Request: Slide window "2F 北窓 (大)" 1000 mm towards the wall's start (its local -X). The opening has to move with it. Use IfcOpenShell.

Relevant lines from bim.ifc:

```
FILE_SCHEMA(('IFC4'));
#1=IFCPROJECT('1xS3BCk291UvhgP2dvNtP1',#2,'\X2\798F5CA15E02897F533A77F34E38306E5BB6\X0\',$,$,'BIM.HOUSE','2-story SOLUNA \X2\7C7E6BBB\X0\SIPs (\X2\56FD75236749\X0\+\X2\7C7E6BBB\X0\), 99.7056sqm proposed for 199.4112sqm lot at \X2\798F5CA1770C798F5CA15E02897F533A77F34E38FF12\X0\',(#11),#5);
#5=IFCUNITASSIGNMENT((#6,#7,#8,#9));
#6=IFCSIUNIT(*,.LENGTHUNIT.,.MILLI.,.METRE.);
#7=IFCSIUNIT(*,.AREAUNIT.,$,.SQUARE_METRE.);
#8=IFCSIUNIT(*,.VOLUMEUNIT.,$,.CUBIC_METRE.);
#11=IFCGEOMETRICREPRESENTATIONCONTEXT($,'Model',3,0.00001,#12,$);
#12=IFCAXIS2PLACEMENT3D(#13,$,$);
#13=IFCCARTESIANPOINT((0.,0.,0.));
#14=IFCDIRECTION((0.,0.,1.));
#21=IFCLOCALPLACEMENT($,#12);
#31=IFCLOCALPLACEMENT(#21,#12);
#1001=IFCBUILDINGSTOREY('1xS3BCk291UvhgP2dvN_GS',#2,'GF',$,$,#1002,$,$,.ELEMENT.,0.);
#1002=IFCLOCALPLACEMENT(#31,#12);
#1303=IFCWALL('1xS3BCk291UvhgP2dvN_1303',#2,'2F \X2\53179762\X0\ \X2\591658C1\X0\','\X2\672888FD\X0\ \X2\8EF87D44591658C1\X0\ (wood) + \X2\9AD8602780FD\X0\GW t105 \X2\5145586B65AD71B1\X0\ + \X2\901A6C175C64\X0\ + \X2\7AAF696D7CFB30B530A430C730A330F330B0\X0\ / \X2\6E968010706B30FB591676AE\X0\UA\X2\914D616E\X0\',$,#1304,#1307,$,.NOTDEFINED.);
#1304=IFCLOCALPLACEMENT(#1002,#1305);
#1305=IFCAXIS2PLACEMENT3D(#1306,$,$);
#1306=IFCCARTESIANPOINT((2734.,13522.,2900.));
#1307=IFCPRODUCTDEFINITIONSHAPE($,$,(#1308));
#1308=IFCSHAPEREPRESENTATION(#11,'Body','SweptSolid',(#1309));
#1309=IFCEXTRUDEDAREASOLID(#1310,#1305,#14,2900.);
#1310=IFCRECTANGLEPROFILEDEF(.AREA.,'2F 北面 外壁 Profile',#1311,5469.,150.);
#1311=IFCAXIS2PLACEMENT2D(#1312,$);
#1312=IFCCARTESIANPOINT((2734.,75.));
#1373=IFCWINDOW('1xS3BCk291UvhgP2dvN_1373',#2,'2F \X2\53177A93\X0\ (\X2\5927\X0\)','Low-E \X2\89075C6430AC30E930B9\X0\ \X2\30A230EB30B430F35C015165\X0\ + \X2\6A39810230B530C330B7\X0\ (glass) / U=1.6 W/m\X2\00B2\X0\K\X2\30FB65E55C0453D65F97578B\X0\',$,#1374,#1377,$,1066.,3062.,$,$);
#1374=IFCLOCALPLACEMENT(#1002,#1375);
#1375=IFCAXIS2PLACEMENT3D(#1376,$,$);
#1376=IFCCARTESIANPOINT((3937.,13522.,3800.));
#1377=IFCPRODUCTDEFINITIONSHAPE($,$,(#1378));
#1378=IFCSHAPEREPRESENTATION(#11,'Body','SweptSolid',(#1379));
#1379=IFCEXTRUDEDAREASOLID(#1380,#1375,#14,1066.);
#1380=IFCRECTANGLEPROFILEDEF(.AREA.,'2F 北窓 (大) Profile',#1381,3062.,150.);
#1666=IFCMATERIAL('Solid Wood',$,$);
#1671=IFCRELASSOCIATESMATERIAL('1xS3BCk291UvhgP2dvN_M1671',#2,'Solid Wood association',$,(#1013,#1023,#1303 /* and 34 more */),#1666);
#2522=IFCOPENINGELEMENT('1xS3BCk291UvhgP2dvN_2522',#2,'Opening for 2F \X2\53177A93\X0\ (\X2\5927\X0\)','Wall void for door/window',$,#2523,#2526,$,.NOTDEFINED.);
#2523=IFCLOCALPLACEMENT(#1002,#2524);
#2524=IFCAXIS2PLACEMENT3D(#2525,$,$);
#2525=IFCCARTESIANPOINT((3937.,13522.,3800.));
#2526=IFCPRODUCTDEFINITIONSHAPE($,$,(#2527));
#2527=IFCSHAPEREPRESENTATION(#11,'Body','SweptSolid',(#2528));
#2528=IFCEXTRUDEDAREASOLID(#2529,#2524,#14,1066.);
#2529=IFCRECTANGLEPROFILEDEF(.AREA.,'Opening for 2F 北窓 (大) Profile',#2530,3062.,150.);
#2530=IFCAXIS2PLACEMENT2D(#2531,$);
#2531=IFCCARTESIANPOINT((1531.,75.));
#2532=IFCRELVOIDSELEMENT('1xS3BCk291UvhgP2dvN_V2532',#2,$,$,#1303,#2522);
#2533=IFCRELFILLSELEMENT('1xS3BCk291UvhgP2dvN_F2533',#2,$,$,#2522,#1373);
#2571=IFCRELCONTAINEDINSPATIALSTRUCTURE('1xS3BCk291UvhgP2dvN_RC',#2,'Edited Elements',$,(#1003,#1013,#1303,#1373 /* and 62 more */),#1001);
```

```python
import ifcopenshell
import ifcopenshell.api.geometry
import ifcopenshell.util.placement
import ifcopenshell.util.unit

model = ifcopenshell.open("bim.ifc")
unit_scale = ifcopenshell.util.unit.calculate_unit_scale(model)

window = model.by_guid("1xS3BCk291UvhgP2dvN_1373")
opening = window.FillsVoids[0].RelatingOpeningElement
wall = opening.VoidsElements[0].RelatingBuildingElement

wall_matrix = ifcopenshell.util.placement.get_local_placement(wall.ObjectPlacement)
shift = wall_matrix[:3, 0] * -1 / unit_scale
before = ifcopenshell.util.placement.get_local_placement(window.ObjectPlacement)[:3, 3].copy()

# The window is not placed relative to its opening, so move both.
for product in (opening, window):
    matrix = ifcopenshell.util.placement.get_local_placement(product.ObjectPlacement)
    matrix[:3, 3] += shift
    ifcopenshell.api.geometry.edit_object_placement(model, product=product, matrix=matrix, is_si=False)

after = ifcopenshell.util.placement.get_local_placement(window.ObjectPlacement)[:3, 3]
print("window moved by", (after - before).round(3) + 0.0)

model.write("bim_edited.ifc")
```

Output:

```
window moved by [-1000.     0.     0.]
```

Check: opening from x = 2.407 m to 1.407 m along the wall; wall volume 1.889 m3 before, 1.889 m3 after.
